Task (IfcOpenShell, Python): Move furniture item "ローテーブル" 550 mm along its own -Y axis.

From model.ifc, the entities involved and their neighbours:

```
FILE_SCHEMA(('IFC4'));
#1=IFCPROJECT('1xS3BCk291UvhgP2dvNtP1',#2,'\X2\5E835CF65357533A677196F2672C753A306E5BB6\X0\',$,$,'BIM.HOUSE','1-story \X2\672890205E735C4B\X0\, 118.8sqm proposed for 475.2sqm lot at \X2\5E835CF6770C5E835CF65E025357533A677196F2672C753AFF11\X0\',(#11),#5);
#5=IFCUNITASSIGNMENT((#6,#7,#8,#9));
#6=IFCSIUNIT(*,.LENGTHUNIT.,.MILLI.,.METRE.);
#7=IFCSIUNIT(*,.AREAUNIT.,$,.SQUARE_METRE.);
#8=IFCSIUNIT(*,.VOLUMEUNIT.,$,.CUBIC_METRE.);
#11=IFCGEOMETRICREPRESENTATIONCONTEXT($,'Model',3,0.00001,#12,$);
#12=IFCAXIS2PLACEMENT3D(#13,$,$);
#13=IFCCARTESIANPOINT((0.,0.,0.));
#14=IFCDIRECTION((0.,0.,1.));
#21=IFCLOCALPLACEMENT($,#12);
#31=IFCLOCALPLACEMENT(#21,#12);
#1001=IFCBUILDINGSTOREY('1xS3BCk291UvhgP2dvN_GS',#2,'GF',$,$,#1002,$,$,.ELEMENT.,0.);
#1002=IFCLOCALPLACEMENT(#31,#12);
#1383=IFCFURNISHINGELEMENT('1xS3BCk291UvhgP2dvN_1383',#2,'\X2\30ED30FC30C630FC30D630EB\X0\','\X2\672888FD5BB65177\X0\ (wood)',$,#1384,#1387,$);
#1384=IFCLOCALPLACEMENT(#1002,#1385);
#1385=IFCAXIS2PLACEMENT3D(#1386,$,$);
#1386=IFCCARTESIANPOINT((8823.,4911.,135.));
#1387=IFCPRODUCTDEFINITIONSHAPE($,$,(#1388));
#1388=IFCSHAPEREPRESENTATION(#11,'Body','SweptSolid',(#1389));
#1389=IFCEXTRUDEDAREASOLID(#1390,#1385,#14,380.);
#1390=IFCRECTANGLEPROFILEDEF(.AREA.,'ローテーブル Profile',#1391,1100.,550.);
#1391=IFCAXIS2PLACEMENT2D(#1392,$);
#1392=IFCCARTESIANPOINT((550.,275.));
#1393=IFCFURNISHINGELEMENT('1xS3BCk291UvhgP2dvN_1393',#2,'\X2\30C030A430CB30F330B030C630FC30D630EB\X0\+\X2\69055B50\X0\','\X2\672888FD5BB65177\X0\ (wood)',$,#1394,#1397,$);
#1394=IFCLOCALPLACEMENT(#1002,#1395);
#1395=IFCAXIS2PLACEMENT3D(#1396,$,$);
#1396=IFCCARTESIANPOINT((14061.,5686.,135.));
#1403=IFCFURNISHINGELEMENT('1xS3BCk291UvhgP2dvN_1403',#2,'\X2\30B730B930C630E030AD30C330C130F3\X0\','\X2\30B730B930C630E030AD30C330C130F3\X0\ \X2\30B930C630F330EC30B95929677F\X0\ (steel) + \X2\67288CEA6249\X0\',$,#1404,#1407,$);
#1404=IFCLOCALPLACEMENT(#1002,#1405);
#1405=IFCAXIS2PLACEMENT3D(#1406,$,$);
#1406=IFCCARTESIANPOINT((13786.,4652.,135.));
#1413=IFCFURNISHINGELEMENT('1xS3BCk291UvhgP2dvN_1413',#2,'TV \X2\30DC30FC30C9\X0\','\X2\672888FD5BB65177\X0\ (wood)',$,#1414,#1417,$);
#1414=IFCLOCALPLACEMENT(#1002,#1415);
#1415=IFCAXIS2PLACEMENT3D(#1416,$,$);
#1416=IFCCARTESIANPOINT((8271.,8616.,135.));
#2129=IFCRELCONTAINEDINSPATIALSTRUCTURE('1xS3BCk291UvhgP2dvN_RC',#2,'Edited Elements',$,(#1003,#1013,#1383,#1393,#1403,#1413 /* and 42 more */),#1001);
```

```python
import ifcopenshell
import ifcopenshell.api.geometry
import ifcopenshell.util.placement
import ifcopenshell.util.unit

model = ifcopenshell.open("model.ifc")
unit_scale = ifcopenshell.util.unit.calculate_unit_scale(model)

item = model.by_id(1383)
matrix = ifcopenshell.util.placement.get_local_placement(item.ObjectPlacement)
matrix[:3, 3] -= matrix[:3, 1] * 0.55 / unit_scale
ifcopenshell.api.geometry.edit_object_placement(model, product=item, matrix=matrix, is_si=False)

print(ifcopenshell.util.placement.get_local_placement(item.ObjectPlacement).round(3) + 0.0)

model.write("model_edited.ifc")
```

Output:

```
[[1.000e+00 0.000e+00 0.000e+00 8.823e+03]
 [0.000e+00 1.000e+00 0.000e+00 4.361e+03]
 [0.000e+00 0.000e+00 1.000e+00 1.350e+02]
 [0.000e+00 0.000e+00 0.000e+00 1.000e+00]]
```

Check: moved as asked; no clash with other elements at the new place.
